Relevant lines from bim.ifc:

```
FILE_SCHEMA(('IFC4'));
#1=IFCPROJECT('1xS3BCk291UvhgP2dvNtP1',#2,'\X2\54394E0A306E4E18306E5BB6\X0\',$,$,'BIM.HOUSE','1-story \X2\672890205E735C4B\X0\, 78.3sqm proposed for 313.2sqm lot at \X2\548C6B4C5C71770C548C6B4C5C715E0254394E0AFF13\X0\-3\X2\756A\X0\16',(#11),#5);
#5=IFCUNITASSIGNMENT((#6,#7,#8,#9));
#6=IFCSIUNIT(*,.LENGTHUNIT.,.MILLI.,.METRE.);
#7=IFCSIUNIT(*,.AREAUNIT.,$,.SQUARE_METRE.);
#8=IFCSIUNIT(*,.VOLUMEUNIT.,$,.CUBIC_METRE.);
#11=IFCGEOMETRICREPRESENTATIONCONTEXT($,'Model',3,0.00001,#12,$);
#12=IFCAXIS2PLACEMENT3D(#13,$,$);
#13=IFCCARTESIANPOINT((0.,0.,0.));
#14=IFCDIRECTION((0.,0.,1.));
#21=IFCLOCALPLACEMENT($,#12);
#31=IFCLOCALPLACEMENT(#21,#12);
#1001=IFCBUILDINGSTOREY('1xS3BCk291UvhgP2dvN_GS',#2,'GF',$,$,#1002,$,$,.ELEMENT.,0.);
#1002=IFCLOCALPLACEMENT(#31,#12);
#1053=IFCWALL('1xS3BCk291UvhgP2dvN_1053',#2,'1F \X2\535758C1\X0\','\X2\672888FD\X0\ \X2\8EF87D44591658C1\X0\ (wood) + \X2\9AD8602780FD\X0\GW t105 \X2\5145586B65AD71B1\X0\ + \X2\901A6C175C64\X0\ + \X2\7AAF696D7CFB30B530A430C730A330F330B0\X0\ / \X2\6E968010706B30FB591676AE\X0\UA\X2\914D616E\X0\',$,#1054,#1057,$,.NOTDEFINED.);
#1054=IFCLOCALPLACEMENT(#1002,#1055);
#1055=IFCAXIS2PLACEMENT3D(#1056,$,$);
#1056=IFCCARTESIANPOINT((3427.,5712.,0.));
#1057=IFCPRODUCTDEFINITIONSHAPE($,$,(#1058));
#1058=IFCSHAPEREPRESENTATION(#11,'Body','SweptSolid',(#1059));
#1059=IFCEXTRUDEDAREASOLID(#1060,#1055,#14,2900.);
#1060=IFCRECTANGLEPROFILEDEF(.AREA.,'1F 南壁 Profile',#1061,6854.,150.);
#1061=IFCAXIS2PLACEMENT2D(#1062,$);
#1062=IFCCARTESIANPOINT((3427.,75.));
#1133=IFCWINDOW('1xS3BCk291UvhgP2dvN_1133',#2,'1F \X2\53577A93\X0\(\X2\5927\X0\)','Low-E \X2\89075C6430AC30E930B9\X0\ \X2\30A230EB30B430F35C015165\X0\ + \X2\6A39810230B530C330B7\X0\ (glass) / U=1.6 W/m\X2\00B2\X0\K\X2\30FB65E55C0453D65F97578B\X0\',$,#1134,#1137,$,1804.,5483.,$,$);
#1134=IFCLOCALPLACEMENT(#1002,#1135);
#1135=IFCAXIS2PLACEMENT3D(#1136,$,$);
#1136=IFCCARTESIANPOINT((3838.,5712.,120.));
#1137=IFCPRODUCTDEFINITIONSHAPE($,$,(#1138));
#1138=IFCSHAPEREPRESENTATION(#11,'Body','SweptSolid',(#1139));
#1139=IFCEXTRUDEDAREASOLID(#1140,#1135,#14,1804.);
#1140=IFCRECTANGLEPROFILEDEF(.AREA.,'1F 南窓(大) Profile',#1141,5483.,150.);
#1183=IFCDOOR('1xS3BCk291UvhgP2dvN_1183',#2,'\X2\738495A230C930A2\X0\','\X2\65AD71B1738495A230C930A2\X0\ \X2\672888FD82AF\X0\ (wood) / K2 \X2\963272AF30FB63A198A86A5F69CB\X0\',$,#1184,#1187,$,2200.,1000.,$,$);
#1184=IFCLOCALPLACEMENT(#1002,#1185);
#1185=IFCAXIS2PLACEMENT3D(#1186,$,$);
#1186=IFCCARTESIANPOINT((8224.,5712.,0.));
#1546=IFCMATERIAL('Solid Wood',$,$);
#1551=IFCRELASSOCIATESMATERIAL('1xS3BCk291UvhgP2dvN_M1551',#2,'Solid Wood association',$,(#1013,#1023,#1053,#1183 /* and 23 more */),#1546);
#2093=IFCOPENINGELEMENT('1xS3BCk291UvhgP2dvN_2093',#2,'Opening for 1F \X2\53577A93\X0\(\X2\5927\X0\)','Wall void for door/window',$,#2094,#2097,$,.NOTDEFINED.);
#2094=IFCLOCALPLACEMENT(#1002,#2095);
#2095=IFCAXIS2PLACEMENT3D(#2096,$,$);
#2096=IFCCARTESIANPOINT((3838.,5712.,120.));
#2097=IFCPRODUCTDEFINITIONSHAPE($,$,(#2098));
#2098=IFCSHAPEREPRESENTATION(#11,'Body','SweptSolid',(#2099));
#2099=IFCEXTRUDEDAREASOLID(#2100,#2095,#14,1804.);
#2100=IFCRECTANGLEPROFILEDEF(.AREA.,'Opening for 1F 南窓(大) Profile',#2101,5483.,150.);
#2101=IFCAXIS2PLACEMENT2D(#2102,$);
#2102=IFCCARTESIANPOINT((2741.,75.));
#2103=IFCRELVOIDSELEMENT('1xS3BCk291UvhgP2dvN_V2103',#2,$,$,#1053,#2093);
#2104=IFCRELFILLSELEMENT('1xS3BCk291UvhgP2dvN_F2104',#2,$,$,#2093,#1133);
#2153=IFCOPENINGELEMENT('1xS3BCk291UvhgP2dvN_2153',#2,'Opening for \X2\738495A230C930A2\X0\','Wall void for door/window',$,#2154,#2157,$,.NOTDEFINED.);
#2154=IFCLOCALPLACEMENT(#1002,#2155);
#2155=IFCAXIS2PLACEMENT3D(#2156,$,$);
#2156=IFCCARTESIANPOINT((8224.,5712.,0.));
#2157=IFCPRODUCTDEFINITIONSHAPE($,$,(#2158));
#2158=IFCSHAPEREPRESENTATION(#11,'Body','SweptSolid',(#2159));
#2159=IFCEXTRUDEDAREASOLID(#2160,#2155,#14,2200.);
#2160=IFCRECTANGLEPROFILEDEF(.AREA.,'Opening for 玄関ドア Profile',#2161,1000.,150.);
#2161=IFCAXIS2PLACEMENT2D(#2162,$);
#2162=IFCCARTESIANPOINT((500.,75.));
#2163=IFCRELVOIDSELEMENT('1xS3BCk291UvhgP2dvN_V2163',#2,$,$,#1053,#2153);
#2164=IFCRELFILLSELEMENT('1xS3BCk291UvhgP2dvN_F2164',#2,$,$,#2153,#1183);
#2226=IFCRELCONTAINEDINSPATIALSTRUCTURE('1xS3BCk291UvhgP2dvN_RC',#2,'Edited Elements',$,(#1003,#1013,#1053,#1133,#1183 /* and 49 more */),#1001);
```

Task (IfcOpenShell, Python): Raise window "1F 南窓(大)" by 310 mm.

```python
import numpy as np
import ifcopenshell
import ifcopenshell.api.geometry
import ifcopenshell.util.placement
import ifcopenshell.util.unit

model = ifcopenshell.open("bim.ifc")
unit_scale = ifcopenshell.util.unit.calculate_unit_scale(model)

window = model.by_id(1133)
opening = window.FillsVoids[0].RelatingOpeningElement
dz = 0.31 / unit_scale

shift = np.array([0.0, 0.0, dz])
# The window is not placed relative to its opening, so move both.
for product in (opening, window):
    matrix = ifcopenshell.util.placement.get_local_placement(product.ObjectPlacement)
    matrix[:3, 3] += shift
    ifcopenshell.api.geometry.edit_object_placement(model, product=product, matrix=matrix, is_si=False)

print(f"moved by {dz * unit_scale:+.3f} m")

model.write("bim_v2.ifc")
```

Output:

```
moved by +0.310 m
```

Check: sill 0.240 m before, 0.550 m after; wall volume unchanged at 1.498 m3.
